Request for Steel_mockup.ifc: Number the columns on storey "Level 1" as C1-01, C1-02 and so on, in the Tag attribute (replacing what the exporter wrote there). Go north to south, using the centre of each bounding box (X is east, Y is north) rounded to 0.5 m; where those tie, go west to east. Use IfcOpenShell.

First a look at what the model holds.

```python
import ifcopenshell
import ifcopenshell.util.element
import ifcopenshell.util.placement

model = ifcopenshell.open("Steel_mockup.ifc")
print(model.schema)
storey = next(s for s in model.by_type("IfcBuildingStorey") if s.Name == "Level 1")
columns = [e for e in ifcopenshell.util.element.get_decomposition(storey) if e.is_a("IfcColumn")]
for e in sorted(columns, key=lambda e: e.id()):
    origin = ifcopenshell.util.placement.get_local_placement(e.ObjectPlacement)[:3, 3]
    print(e.id(), e.Tag, e.Name, origin.round(2) + 0.0, sep=" | ")
```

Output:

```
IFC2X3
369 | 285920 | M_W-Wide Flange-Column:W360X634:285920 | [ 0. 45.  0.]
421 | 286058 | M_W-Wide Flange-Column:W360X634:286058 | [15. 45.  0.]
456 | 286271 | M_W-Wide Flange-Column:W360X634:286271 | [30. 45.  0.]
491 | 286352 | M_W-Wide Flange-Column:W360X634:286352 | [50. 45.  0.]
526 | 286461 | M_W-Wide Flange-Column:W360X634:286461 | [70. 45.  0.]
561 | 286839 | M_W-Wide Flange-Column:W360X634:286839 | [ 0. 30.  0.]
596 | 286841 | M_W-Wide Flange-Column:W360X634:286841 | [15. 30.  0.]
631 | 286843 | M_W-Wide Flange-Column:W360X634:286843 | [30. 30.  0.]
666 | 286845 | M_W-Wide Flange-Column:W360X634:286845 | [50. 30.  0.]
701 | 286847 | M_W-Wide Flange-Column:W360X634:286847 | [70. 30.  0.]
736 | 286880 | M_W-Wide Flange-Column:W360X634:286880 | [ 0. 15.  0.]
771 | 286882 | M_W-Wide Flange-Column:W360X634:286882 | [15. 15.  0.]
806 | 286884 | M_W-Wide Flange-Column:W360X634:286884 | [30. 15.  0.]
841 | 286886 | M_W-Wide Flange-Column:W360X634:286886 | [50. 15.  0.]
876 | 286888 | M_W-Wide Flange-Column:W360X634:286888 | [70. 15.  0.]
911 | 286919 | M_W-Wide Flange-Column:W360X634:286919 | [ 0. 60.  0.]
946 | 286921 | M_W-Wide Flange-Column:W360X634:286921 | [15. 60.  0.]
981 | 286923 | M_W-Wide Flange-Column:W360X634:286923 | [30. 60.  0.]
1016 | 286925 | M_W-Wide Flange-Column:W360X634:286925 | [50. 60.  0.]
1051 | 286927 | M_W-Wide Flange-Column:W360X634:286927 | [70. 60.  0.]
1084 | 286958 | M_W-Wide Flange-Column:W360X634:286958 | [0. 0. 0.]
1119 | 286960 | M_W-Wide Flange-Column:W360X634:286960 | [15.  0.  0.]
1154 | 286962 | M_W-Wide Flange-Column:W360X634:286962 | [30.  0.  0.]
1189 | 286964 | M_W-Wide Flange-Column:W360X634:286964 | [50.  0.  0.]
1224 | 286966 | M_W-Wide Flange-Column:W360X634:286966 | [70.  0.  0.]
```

```python
import ifcopenshell
import ifcopenshell.geom
import ifcopenshell.util.element
import ifcopenshell.util.shape

model = ifcopenshell.open("Steel_mockup.ifc")
settings = ifcopenshell.geom.settings()
settings.set("use-world-coords", True)


def centre(element):
    shape = ifcopenshell.geom.create_shape(settings, element)
    return ifcopenshell.util.shape.get_bbox_centroid(shape.geometry)


storey = next(s for s in model.by_type("IfcBuildingStorey") if s.Name == "Level 1")
columns = [e for e in ifcopenshell.util.element.get_decomposition(storey) if e.is_a("IfcColumn")]

# Insertion points can sit at a corner or the storey origin, so sort by the geometry (in metres).
centres = {e: centre(e) for e in columns}
columns.sort(key=lambda e: (-round(centres[e][1] / 0.5), centres[e][0]))

for i, e in enumerate(columns, start=1):
    number = f"C1-{i:02d}"
    e.Tag = number
    print(e.id(), number)

model.write("Steel_mockup_edited.ifc")
```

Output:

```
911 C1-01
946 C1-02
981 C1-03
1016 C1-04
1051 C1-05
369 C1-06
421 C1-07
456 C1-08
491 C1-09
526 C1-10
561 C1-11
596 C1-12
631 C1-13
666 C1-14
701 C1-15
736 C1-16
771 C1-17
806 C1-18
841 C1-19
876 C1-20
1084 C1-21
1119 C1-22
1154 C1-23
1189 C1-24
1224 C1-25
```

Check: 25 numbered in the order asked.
